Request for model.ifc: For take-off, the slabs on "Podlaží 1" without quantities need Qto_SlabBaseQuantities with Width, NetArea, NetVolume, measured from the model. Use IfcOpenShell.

First a look at what the model holds.

```python
import ifcopenshell
import ifcopenshell.util.element
import ifcopenshell.util.unit

model = ifcopenshell.open("model.ifc")
print(model.schema)
for unit_type in ("LENGTHUNIT", "AREAUNIT", "VOLUMEUNIT"):
    print(unit_type, ifcopenshell.util.unit.calculate_unit_scale(model, unit_type))
storey = next(s for s in model.by_type("IfcBuildingStorey") if s.Name == "Podlaží 1")
slabs = [e for e in ifcopenshell.util.element.get_decomposition(storey) if e.is_a("IfcSlab")]
for e in sorted(slabs, key=lambda e: e.id()):
    print(e.id(), e.is_a(), e.Name, list(ifcopenshell.util.element.get_psets(e, qtos_only=True)), sep=" | ")
```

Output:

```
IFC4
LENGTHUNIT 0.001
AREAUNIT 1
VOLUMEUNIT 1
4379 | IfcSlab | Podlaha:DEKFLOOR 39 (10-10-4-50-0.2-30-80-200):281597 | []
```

```python
import ifcopenshell
import ifcopenshell.api.pset
import ifcopenshell.geom
import ifcopenshell.util.element
import ifcopenshell.util.shape
import ifcopenshell.util.unit

model = ifcopenshell.open("model.ifc")
unit_scale = ifcopenshell.util.unit.calculate_unit_scale(model)
area_scale = ifcopenshell.util.unit.calculate_unit_scale(model, "AREAUNIT")
volume_scale = ifcopenshell.util.unit.calculate_unit_scale(model, "VOLUMEUNIT")
settings = ifcopenshell.geom.settings()

storey = next(s for s in model.by_type("IfcBuildingStorey") if s.Name == "Podlaží 1")
slabs = [e for e in ifcopenshell.util.element.get_decomposition(storey) if e.is_a("IfcSlab")]

for e in sorted(slabs, key=lambda e: e.id()):
    if ifcopenshell.util.element.get_psets(e, qtos_only=True, should_inherit=False):
        continue
    # Geometry comes back in metres, in the element's own axes.
    shape = ifcopenshell.geom.create_shape(settings, e)
    values = {
        "Width": ifcopenshell.util.shape.get_z(shape.geometry) / unit_scale,
        "NetArea": ifcopenshell.util.shape.get_footprint_area(shape.geometry) / area_scale,
        "NetVolume": ifcopenshell.util.shape.get_volume(shape.geometry) / volume_scale,
    }
    qto = ifcopenshell.api.pset.add_qto(model, product=e, name="Qto_SlabBaseQuantities")
    ifcopenshell.api.pset.edit_qto(model, qto=qto, properties=values)
    print(e.id(), {k: round(v, 3) for k, v in values.items()})

model.write("model_v2.ifc")
```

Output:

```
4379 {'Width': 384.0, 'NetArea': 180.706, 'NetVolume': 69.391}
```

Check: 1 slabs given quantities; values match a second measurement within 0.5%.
